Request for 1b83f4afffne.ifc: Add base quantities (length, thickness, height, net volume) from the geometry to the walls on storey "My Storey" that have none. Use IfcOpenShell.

First a look at what the model holds.

```python
import ifcopenshell
import ifcopenshell.util.element
import ifcopenshell.util.unit

model = ifcopenshell.open("1b83f4afffne.ifc")
print(model.schema)
for unit_type in ("LENGTHUNIT", "AREAUNIT", "VOLUMEUNIT"):
    print(unit_type, ifcopenshell.util.unit.calculate_unit_scale(model, unit_type))
storey = next(s for s in model.by_type("IfcBuildingStorey") if s.Name == "My Storey")
walls = [e for e in ifcopenshell.util.element.get_decomposition(storey) if e.is_a("IfcWall")]
for e in sorted(walls, key=lambda e: e.id()):
    print(e.id(), e.is_a(), e.Name, list(ifcopenshell.util.element.get_psets(e, qtos_only=True)), sep=" | ")
```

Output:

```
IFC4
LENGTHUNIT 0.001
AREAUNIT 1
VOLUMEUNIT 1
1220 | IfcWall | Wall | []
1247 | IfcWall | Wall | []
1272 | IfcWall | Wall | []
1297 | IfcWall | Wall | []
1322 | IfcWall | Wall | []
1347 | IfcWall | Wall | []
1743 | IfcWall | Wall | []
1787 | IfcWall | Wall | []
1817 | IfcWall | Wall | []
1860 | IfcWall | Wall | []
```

```python
import ifcopenshell
import ifcopenshell.api.pset
import ifcopenshell.geom
import ifcopenshell.util.element
import ifcopenshell.util.shape
import ifcopenshell.util.unit

model = ifcopenshell.open("1b83f4afffne.ifc")
unit_scale = ifcopenshell.util.unit.calculate_unit_scale(model)
volume_scale = ifcopenshell.util.unit.calculate_unit_scale(model, "VOLUMEUNIT")
settings = ifcopenshell.geom.settings()

storey = next(s for s in model.by_type("IfcBuildingStorey") if s.Name == "My Storey")
walls = [e for e in ifcopenshell.util.element.get_decomposition(storey) if e.is_a("IfcWall")]

for e in sorted(walls, key=lambda e: e.id()):
    if ifcopenshell.util.element.get_psets(e, qtos_only=True, should_inherit=False):
        continue
    # Geometry comes back in metres, in the element's own axes.
    shape = ifcopenshell.geom.create_shape(settings, e)
    values = {
        "Length": ifcopenshell.util.shape.get_x(shape.geometry) / unit_scale,
        "Width": ifcopenshell.util.shape.get_y(shape.geometry) / unit_scale,
        "Height": ifcopenshell.util.shape.get_z(shape.geometry) / unit_scale,
        "NetVolume": ifcopenshell.util.shape.get_volume(shape.geometry) / volume_scale,
    }
    qto = ifcopenshell.api.pset.add_qto(model, product=e, name="Qto_WallBaseQuantities")
    ifcopenshell.api.pset.edit_qto(model, qto=qto, properties=values)
    print(e.id(), {k: round(v, 3) for k, v in values.items()})

model.write("1b83f4afffne_updated.ifc")
```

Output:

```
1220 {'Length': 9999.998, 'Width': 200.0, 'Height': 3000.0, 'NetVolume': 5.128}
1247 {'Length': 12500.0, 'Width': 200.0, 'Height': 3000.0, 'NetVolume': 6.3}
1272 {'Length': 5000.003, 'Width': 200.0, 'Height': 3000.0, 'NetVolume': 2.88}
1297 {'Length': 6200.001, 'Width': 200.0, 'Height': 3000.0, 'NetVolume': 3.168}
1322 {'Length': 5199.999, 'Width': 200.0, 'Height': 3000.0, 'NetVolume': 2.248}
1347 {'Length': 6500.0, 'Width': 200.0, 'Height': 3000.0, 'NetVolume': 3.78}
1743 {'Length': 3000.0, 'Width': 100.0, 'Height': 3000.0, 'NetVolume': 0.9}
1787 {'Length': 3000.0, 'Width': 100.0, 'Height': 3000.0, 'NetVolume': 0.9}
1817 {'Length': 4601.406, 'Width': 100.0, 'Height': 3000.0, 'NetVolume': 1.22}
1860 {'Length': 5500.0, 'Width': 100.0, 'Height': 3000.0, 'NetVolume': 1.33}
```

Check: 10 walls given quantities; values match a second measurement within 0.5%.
